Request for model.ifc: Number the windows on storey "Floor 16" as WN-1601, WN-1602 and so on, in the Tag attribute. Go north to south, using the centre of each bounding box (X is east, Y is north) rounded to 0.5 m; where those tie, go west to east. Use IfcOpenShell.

First a look at what the model holds.

```python
import ifcopenshell
import ifcopenshell.util.element
import ifcopenshell.util.placement

model = ifcopenshell.open("model.ifc")
print(model.schema)
storey = next(s for s in model.by_type("IfcBuildingStorey") if s.Name == "Floor 16")
windows = [e for e in ifcopenshell.util.element.get_decomposition(storey) if e.is_a("IfcWindow")]
for e in sorted(windows, key=lambda e: e.id()):
    origin = ifcopenshell.util.placement.get_local_placement(e.ObjectPlacement)[:3, 3]
    print(e.id(), e.Tag, e.Name, origin.round(2) + 0.0, sep=" | ")
```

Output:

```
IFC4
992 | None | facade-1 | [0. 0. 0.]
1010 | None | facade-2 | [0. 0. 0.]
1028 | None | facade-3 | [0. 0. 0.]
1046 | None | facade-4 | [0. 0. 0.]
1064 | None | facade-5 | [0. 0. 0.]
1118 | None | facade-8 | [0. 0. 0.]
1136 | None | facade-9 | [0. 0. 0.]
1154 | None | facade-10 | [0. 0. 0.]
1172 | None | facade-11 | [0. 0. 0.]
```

```python
import ifcopenshell
import ifcopenshell.geom
import ifcopenshell.util.element
import ifcopenshell.util.shape

model = ifcopenshell.open("model.ifc")
settings = ifcopenshell.geom.settings()
settings.set("use-world-coords", True)


def centre(element):
    shape = ifcopenshell.geom.create_shape(settings, element)
    return ifcopenshell.util.shape.get_bbox_centroid(shape.geometry)


storey = next(s for s in model.by_type("IfcBuildingStorey") if s.Name == "Floor 16")
windows = [e for e in ifcopenshell.util.element.get_decomposition(storey) if e.is_a("IfcWindow")]

# Insertion points can sit at a corner or the storey origin, so sort by the geometry (in metres).
centres = {e: centre(e) for e in windows}
windows.sort(key=lambda e: (-round(centres[e][1] / 0.5), centres[e][0]))

for i, e in enumerate(windows, start=1):
    number = f"WN-16{i:02d}"
    e.Tag = number
    print(e.id(), number)

model.write("model-out.ifc")
```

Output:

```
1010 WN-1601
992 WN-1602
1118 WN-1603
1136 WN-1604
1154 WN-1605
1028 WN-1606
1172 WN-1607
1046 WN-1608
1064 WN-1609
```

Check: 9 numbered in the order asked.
